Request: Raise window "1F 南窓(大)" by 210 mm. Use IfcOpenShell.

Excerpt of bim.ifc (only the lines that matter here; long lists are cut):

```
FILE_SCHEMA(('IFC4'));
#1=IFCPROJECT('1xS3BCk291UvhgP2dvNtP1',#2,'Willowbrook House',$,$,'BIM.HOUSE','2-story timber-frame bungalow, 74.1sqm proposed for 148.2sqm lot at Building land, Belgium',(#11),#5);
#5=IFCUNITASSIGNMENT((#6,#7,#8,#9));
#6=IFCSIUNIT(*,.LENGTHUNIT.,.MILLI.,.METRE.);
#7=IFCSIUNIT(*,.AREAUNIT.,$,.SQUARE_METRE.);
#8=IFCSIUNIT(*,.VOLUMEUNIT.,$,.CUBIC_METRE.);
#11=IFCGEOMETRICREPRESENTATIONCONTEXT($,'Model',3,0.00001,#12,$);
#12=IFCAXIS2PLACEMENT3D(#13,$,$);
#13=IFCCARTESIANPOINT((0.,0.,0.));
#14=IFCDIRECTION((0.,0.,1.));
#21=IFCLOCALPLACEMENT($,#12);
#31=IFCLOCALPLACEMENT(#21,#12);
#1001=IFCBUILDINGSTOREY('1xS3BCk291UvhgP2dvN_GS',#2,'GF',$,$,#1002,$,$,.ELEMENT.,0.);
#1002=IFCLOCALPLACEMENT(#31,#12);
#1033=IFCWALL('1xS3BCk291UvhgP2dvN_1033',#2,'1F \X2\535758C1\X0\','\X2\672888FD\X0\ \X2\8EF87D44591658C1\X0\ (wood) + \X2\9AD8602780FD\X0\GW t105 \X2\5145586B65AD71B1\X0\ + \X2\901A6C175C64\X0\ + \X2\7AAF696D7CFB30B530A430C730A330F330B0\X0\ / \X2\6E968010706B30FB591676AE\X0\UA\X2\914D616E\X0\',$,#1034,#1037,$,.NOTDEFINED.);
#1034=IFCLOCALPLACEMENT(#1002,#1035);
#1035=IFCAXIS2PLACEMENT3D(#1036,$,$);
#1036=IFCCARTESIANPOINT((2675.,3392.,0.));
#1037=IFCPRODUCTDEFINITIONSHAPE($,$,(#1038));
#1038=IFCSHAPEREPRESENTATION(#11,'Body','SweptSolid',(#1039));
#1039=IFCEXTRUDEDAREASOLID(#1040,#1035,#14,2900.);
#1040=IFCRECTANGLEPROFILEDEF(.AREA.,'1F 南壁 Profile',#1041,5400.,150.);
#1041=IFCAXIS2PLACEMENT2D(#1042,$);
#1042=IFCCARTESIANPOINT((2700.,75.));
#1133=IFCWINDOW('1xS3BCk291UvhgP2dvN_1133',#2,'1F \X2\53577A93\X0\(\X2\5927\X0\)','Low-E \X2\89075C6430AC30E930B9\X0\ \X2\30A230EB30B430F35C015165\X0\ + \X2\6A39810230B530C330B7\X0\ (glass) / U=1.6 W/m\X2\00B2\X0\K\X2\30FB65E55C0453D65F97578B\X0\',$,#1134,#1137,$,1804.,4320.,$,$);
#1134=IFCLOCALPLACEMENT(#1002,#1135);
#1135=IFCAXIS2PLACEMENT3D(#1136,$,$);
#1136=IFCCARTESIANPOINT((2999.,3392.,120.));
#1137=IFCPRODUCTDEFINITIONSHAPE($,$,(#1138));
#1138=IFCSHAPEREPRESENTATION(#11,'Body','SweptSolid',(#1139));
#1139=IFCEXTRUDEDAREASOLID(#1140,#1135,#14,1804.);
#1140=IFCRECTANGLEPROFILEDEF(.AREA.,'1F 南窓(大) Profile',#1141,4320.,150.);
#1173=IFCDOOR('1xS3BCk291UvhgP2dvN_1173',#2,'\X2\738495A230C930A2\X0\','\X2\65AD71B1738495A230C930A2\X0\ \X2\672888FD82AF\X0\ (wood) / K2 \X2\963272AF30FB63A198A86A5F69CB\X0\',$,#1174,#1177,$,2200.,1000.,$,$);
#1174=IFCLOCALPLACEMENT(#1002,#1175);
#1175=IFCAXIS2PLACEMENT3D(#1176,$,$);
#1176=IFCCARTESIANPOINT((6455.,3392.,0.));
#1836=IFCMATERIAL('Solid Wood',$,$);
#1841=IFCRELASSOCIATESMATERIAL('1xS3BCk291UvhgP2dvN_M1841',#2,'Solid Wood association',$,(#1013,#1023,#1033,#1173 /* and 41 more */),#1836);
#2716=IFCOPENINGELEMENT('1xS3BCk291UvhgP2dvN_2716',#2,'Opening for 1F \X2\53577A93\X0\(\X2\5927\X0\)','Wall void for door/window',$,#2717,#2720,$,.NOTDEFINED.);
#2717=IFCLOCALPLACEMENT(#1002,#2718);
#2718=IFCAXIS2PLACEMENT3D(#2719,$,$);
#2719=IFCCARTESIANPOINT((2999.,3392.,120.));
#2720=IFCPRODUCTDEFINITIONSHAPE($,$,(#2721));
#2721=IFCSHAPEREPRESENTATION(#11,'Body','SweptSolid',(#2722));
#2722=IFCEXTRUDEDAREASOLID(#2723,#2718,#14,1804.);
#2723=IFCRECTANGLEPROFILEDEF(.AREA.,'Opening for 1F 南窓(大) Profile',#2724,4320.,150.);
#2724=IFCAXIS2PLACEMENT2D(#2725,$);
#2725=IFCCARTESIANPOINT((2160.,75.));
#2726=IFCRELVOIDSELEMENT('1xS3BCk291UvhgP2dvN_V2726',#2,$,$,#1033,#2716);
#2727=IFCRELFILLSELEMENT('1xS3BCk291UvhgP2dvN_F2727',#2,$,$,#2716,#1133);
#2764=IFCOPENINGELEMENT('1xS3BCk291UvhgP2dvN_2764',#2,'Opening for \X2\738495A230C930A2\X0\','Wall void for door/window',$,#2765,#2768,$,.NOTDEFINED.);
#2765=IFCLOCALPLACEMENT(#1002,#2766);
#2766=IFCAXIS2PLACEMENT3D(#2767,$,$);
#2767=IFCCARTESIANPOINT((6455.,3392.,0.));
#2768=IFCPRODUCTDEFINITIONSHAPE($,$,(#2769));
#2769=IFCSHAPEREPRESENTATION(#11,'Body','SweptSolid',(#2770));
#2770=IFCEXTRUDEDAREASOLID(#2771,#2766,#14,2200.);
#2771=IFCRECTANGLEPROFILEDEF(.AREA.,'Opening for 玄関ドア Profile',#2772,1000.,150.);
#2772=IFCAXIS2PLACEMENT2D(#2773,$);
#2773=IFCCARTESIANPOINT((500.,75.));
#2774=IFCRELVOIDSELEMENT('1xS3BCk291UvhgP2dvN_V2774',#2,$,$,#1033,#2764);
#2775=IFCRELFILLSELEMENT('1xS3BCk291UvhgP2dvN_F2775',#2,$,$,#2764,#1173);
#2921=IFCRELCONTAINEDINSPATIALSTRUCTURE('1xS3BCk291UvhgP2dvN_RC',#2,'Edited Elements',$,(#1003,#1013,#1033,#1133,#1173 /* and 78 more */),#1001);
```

```python
import numpy as np
import ifcopenshell
import ifcopenshell.api.geometry
import ifcopenshell.util.placement
import ifcopenshell.util.unit

model = ifcopenshell.open("bim.ifc")
unit_scale = ifcopenshell.util.unit.calculate_unit_scale(model)

window = model.by_guid("1xS3BCk291UvhgP2dvN_1133")
opening = window.FillsVoids[0].RelatingOpeningElement
dz = 0.21 / unit_scale

shift = np.array([0.0, 0.0, dz])
# The window is not placed relative to its opening, so move both.
for product in (opening, window):
    matrix = ifcopenshell.util.placement.get_local_placement(product.ObjectPlacement)
    matrix[:3, 3] += shift
    ifcopenshell.api.geometry.edit_object_placement(model, product=product, matrix=matrix, is_si=False)

print(f"moved by {dz * unit_scale:+.3f} m")

model.write("bim_updated.ifc")
```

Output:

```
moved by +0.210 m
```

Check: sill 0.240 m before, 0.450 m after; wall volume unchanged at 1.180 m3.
